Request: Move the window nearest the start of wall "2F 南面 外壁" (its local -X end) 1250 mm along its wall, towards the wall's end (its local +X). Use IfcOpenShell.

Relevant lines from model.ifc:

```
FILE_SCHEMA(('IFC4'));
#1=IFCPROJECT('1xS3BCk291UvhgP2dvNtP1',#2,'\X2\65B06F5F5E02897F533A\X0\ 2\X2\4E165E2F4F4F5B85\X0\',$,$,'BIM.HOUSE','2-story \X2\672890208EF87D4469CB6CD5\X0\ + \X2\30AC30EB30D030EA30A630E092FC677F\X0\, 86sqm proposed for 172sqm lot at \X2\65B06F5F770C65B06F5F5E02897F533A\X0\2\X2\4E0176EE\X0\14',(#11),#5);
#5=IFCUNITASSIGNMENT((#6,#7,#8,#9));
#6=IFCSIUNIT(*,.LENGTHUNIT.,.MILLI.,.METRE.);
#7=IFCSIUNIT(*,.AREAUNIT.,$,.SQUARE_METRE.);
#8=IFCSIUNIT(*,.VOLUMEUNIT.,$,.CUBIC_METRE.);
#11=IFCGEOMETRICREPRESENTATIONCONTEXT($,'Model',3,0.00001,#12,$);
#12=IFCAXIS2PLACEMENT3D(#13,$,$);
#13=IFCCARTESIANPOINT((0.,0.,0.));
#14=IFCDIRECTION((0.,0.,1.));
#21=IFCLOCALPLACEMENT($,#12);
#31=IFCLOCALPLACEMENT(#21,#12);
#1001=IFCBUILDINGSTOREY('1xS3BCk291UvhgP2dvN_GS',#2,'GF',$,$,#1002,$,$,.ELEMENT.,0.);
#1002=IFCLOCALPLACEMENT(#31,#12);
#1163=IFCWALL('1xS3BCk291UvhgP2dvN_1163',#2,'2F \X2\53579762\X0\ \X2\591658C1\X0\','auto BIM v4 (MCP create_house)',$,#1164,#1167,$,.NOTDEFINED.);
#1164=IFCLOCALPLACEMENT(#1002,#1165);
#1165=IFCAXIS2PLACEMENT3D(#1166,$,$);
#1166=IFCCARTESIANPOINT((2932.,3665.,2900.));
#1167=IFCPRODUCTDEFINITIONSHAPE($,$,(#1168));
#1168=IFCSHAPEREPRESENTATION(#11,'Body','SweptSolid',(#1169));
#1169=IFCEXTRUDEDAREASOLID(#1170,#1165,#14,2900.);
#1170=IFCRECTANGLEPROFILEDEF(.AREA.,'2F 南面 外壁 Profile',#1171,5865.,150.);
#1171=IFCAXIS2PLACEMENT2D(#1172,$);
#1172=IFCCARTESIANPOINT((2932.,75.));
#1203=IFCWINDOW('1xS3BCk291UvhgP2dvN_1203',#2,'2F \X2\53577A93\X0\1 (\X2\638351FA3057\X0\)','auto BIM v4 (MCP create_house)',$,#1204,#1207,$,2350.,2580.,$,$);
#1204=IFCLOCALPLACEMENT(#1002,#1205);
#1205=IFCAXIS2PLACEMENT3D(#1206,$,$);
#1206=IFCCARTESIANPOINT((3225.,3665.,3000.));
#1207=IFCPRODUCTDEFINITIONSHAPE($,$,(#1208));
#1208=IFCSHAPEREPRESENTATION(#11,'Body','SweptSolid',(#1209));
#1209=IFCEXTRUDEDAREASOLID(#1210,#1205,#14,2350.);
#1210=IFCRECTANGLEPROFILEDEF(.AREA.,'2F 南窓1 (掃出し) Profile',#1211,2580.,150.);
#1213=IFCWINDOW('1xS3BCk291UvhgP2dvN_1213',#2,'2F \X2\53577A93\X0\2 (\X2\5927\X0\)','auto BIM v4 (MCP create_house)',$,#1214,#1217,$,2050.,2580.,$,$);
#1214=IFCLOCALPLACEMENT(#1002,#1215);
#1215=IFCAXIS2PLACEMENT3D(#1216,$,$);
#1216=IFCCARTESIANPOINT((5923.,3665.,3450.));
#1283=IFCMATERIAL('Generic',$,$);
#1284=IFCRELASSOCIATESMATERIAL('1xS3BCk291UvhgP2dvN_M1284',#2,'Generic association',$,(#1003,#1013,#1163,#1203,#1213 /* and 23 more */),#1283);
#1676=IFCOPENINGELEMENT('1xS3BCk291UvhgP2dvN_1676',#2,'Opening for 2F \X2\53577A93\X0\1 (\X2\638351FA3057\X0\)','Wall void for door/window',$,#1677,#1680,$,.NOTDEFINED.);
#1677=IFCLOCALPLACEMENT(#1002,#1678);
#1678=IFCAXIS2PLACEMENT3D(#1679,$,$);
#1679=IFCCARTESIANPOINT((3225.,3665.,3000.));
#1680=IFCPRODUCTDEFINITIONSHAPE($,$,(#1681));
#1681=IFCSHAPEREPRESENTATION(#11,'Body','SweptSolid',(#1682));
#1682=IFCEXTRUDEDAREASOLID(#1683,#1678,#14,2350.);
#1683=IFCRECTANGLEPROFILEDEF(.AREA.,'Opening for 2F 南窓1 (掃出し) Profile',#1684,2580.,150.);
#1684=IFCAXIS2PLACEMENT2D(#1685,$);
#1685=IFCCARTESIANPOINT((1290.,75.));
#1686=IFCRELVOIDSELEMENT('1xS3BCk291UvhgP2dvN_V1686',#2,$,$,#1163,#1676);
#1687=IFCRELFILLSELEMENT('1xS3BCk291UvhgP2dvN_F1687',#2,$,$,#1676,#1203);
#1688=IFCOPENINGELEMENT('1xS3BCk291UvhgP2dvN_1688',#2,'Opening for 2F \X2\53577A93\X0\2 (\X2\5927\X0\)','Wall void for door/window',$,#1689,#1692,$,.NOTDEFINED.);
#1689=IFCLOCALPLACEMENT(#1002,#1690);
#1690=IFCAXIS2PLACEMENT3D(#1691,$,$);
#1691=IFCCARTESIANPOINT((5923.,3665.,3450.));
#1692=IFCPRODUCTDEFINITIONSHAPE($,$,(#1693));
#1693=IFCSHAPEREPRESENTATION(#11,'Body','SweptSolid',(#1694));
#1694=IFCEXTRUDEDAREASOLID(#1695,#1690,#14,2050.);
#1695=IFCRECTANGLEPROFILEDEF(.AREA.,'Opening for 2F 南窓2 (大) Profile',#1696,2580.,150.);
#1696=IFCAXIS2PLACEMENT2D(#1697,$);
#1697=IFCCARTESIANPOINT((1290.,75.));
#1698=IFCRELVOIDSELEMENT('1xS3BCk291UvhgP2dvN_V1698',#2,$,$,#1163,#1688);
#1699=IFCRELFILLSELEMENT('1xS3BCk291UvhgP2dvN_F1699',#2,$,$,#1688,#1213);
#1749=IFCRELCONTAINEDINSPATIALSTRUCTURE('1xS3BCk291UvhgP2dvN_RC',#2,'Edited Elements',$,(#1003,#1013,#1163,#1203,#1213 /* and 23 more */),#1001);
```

```python
import ifcopenshell
import ifcopenshell.api.geometry
import ifcopenshell.util.placement
import ifcopenshell.util.unit

model = ifcopenshell.open("model.ifc")
unit_scale = ifcopenshell.util.unit.calculate_unit_scale(model)

window = model.by_guid("1xS3BCk291UvhgP2dvN_1203")
opening = window.FillsVoids[0].RelatingOpeningElement
wall = opening.VoidsElements[0].RelatingBuildingElement

wall_matrix = ifcopenshell.util.placement.get_local_placement(wall.ObjectPlacement)
shift = wall_matrix[:3, 0] * 1.25 / unit_scale
before = ifcopenshell.util.placement.get_local_placement(window.ObjectPlacement)[:3, 3].copy()

# The window is not placed relative to its opening, so move both.
for product in (opening, window):
    matrix = ifcopenshell.util.placement.get_local_placement(product.ObjectPlacement)
    matrix[:3, 3] += shift
    ifcopenshell.api.geometry.edit_object_placement(model, product=product, matrix=matrix, is_si=False)

after = ifcopenshell.util.placement.get_local_placement(window.ObjectPlacement)[:3, 3]
print("window moved by", (after - before).round(3) + 0.0)

model.write("model_rev.ifc")
```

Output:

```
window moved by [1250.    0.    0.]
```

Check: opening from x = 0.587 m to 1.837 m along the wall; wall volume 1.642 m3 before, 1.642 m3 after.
